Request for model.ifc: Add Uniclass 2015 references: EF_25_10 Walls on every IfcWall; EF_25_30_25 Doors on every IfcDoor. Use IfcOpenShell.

First a look at what the model holds.

```python
import ifcopenshell

model = ifcopenshell.open("model.ifc")
print(model.schema)
print("classifications:", [c.Name for c in model.by_type("IfcClassification")])
for ifc_class in ("IfcDoor", "IfcRoof", "IfcStair", "IfcWall", "IfcWindow"):
    print(ifc_class, len(model.by_type(ifc_class)))
```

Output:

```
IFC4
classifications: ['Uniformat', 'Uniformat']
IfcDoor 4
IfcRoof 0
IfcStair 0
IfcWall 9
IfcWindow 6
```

```python
import ifcopenshell
import ifcopenshell.api.classification

model = ifcopenshell.open("model.ifc")

system = ifcopenshell.api.classification.add_classification(model, classification="Uniclass 2015")

codes = {
    "IfcWall": ("EF_25_10", "Walls"),
    "IfcDoor": ("EF_25_30_25", "Doors"),
}
for ifc_class, (code, name) in codes.items():
    products = model.by_type(ifc_class)
    ifcopenshell.api.classification.add_reference(
        model, products=products, classification=system, identification=code, name=name
    )
    print(code, len(products))

model.write("model_v2.ifc")
```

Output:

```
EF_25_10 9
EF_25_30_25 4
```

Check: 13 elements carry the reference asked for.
